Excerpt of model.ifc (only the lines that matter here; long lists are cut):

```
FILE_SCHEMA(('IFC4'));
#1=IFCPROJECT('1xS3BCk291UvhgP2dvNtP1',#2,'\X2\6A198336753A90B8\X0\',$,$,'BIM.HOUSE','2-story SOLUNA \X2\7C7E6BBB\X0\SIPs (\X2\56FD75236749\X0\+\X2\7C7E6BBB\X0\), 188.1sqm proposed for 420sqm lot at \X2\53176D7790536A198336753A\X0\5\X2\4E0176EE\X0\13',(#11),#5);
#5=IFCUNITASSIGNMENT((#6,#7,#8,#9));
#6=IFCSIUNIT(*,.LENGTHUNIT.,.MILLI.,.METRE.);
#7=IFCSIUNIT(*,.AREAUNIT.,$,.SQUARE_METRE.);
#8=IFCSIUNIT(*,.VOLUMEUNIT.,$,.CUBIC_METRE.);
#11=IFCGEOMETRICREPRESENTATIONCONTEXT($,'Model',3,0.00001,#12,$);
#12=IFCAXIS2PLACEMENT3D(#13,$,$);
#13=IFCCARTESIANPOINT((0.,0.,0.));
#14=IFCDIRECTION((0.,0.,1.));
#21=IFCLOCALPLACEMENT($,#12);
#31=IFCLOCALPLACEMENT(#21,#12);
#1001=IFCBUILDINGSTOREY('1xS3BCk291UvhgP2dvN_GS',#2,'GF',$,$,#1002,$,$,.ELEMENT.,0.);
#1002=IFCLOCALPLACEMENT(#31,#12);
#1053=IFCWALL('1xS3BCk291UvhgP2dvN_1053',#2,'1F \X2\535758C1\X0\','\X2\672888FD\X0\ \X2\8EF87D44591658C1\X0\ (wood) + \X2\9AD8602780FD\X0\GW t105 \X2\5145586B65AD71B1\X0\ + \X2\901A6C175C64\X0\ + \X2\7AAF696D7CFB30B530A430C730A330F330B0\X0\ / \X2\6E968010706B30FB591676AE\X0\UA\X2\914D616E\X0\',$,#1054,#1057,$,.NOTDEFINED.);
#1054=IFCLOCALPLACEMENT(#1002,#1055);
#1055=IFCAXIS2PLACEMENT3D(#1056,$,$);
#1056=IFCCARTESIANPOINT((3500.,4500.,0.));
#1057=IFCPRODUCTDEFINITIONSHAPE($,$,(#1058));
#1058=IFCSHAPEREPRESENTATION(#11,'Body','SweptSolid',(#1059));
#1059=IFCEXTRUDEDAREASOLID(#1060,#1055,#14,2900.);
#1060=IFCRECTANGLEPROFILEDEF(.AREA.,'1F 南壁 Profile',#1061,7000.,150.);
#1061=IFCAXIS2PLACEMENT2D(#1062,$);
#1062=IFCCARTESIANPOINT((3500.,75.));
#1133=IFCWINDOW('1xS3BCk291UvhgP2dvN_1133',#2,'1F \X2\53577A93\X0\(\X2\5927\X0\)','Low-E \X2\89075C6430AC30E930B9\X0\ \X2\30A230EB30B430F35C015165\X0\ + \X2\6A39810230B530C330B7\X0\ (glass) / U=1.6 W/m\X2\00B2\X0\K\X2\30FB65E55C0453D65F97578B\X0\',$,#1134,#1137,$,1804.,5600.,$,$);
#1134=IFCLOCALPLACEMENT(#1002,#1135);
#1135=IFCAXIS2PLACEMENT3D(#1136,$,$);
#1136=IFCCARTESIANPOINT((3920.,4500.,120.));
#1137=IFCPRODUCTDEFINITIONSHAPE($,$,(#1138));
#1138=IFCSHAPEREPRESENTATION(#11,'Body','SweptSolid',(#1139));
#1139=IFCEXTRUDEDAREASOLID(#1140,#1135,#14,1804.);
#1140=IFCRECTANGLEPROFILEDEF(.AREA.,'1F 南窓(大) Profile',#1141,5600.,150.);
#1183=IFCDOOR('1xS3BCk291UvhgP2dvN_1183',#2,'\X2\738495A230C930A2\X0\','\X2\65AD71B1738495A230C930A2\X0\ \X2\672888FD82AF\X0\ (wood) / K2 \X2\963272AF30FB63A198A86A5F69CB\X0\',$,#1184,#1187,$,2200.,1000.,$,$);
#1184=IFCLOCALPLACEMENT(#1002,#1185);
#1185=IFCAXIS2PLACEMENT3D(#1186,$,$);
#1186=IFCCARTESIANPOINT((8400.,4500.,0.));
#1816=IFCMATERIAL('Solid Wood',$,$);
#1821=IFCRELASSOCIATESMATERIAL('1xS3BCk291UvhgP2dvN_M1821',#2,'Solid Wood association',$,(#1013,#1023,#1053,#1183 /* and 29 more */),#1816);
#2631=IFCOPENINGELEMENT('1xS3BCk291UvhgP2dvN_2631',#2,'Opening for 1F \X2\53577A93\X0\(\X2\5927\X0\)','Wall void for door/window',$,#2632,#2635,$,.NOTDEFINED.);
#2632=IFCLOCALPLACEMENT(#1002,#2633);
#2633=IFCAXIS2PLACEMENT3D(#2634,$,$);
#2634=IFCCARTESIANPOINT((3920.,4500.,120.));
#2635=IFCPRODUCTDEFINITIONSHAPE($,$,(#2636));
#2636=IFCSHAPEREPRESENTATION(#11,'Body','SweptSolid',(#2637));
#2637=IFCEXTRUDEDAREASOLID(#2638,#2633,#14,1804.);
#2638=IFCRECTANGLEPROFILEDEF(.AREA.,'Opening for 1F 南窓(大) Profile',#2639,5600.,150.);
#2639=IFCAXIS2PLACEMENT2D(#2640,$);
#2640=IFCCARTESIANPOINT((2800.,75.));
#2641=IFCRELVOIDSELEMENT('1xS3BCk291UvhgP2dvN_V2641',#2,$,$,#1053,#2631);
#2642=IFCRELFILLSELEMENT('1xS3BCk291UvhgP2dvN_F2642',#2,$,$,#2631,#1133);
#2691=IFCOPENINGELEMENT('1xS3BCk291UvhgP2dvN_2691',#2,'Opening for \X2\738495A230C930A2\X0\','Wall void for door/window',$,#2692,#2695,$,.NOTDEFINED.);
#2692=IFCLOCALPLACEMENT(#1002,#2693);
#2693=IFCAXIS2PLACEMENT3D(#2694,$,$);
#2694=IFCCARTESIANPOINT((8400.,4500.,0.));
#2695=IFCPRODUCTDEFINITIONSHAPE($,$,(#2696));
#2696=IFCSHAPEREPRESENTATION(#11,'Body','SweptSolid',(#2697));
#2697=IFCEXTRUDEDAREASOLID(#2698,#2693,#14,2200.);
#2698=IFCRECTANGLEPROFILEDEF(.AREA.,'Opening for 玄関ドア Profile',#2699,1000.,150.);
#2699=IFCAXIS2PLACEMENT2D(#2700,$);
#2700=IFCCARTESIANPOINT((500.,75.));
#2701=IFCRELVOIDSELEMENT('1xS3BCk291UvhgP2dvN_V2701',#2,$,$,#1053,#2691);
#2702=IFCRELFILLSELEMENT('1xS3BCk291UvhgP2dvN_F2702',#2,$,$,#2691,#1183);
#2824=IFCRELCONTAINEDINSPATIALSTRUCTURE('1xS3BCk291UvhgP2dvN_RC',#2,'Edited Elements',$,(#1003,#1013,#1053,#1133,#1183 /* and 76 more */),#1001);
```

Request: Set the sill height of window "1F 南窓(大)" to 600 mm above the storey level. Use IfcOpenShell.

```python
import numpy as np
import ifcopenshell
import ifcopenshell.api.geometry
import ifcopenshell.geom
import ifcopenshell.util.element
import ifcopenshell.util.placement
import ifcopenshell.util.shape
import ifcopenshell.util.unit

model = ifcopenshell.open("model.ifc")
unit_scale = ifcopenshell.util.unit.calculate_unit_scale(model)

window = model.by_guid("1xS3BCk291UvhgP2dvN_1133")
opening = window.FillsVoids[0].RelatingOpeningElement
storey = ifcopenshell.util.element.get_container(window, ifc_class="IfcBuildingStorey")
level = ifcopenshell.util.placement.get_local_placement(storey.ObjectPlacement)[2, 3]

# The opening's origin need not be at the sill, so measure its lowest point.
shape = ifcopenshell.geom.create_shape(ifcopenshell.geom.settings(), opening)
bottom = ifcopenshell.util.shape.get_shape_bottom_elevation(shape, shape.geometry) / unit_scale
dz = level + 600.0 - bottom

shift = np.array([0.0, 0.0, dz])
# The window is not placed relative to its opening, so move both.
for product in (opening, window):
    matrix = ifcopenshell.util.placement.get_local_placement(product.ObjectPlacement)
    matrix[:3, 3] += shift
    ifcopenshell.api.geometry.edit_object_placement(model, product=product, matrix=matrix, is_si=False)

print(f"moved by {dz * unit_scale:+.3f} m")

model.write("model_updated.ifc")
```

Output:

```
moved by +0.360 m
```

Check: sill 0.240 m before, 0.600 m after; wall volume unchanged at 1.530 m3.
